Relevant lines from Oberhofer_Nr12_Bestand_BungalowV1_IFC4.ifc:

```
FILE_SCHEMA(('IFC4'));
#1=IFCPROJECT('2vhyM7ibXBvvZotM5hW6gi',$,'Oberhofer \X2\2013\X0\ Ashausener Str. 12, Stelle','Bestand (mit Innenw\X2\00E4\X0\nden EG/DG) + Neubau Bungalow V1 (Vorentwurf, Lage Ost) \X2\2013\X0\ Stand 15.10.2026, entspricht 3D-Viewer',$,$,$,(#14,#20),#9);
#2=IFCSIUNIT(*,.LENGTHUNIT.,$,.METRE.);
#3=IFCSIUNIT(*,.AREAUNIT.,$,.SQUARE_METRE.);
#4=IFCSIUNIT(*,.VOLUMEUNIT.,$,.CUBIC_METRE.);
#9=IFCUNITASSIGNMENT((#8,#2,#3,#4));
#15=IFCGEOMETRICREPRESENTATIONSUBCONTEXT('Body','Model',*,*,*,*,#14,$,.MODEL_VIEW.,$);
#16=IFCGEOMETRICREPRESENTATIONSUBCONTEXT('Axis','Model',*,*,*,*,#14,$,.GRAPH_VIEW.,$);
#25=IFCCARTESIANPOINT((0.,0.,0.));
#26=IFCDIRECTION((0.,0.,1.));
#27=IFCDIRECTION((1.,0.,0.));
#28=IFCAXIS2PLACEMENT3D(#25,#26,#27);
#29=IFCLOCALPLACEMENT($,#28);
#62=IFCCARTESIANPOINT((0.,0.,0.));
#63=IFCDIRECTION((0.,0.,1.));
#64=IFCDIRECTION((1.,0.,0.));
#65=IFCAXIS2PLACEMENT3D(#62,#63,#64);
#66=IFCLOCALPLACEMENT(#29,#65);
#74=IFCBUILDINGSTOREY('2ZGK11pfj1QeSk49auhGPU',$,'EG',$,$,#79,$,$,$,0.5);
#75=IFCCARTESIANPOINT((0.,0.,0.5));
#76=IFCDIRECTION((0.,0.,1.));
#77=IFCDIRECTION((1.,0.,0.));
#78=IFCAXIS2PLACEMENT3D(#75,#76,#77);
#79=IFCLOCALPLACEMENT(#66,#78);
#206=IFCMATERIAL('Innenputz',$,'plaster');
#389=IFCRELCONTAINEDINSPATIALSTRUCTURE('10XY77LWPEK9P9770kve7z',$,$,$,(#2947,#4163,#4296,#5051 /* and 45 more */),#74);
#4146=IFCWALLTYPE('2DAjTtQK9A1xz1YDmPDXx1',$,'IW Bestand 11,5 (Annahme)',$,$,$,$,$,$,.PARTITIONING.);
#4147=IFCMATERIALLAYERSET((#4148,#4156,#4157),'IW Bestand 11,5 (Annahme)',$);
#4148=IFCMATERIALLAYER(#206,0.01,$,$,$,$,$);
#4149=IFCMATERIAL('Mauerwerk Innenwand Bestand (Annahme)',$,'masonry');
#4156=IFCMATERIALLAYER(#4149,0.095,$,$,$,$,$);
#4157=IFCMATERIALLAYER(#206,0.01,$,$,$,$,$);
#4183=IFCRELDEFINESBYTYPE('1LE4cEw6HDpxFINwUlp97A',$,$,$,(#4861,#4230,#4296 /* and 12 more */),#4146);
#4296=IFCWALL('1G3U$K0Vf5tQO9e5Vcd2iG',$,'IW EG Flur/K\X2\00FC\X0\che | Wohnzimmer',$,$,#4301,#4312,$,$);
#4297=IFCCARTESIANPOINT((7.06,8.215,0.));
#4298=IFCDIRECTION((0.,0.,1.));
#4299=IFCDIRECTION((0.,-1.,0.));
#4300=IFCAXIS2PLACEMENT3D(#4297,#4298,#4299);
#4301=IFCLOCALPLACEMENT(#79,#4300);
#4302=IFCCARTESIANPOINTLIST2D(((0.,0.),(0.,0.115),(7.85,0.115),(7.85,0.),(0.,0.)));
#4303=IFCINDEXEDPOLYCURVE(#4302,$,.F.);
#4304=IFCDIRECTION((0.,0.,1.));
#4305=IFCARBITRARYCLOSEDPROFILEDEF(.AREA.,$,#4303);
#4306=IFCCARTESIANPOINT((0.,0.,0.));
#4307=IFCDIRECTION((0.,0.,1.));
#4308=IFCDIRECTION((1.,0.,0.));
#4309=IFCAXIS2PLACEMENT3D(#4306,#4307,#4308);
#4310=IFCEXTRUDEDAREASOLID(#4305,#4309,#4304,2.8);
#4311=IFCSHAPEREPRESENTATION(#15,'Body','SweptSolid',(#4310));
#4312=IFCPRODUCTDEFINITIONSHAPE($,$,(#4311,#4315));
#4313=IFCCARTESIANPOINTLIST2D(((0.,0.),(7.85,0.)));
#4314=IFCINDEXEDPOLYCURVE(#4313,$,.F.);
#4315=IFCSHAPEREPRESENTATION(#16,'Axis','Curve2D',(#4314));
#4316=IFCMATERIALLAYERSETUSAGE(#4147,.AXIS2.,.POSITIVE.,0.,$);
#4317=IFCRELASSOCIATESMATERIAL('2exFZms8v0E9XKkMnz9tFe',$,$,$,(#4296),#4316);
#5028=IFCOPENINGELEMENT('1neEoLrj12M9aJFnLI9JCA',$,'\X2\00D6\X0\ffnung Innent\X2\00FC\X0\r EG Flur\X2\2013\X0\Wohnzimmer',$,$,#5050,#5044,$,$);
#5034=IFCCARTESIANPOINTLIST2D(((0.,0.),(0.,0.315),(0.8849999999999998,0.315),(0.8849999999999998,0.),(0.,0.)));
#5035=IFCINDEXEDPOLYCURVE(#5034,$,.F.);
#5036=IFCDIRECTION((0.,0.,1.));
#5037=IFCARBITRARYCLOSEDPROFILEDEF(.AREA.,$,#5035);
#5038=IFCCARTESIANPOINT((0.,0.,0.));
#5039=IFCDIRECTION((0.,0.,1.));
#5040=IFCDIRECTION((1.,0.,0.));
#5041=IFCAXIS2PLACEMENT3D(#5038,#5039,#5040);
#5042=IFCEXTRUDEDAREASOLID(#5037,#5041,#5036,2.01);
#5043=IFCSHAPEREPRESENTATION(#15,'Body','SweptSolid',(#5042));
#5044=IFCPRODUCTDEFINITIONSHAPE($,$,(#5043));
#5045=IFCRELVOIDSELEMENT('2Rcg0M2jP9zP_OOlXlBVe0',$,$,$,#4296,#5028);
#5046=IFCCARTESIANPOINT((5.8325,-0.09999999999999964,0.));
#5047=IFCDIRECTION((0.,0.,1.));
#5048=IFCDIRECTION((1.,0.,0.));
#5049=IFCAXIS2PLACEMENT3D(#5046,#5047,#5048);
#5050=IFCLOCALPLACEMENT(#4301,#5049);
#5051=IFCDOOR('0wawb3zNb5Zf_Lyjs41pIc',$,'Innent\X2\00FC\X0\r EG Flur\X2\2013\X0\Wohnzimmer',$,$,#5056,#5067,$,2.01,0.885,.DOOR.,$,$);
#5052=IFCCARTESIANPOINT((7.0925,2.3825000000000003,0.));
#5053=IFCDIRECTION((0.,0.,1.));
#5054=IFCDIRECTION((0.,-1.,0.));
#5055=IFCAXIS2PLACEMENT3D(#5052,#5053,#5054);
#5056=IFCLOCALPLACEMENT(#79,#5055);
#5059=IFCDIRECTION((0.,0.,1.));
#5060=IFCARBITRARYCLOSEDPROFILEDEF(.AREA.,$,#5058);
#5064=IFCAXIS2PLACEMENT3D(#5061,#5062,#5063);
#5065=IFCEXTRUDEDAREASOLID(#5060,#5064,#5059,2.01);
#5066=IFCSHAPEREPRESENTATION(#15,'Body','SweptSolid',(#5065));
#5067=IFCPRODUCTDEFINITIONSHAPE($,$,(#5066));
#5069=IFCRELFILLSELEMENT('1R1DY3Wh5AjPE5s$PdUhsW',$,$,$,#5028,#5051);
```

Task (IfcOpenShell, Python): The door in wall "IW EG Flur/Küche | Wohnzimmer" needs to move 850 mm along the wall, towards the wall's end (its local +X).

```python
import ifcopenshell
import ifcopenshell.api.geometry
import ifcopenshell.util.placement
import ifcopenshell.util.unit

model = ifcopenshell.open("Oberhofer_Nr12_Bestand_BungalowV1_IFC4.ifc")
unit_scale = ifcopenshell.util.unit.calculate_unit_scale(model)

door = model.by_guid("0wawb3zNb5Zf_Lyjs41pIc")
opening = door.FillsVoids[0].RelatingOpeningElement
wall = opening.VoidsElements[0].RelatingBuildingElement

wall_matrix = ifcopenshell.util.placement.get_local_placement(wall.ObjectPlacement)
shift = wall_matrix[:3, 0] * 0.85 / unit_scale
before = ifcopenshell.util.placement.get_local_placement(door.ObjectPlacement)[:3, 3].copy()

# The door is not placed relative to its opening, so move both.
for product in (opening, door):
    matrix = ifcopenshell.util.placement.get_local_placement(product.ObjectPlacement)
    matrix[:3, 3] += shift
    ifcopenshell.api.geometry.edit_object_placement(model, product=product, matrix=matrix, is_si=False)

after = ifcopenshell.util.placement.get_local_placement(door.ObjectPlacement)[:3, 3]
print("door moved by", (after - before).round(3) + 0.0)

model.write("Oberhofer_Nr12_Bestand_BungalowV1_IFC4-out.ifc")
```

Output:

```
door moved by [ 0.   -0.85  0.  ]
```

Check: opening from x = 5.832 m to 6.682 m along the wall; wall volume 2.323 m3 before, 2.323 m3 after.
